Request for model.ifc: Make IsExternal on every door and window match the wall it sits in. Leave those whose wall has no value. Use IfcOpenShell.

First a look at what the model holds.

```python
import ifcopenshell
import ifcopenshell.util.element

model = ifcopenshell.open("model.ifc")
print(model.schema)
seen = {}
for e in model.by_type("IfcDoor") + model.by_type("IfcWindow"):
    if not e.FillsVoids:
        continue
    host = e.FillsVoids[0].RelatingOpeningElement.VoidsElements[0].RelatingBuildingElement
    own = ifcopenshell.util.element.get_pset(e, f"Pset_{e.is_a()[3:].removesuffix('StandardCase')}Common", "IsExternal")
    wall = ifcopenshell.util.element.get_pset(host, "Pset_WallCommon", "IsExternal")
    seen[e.is_a(), own, wall] = seen.get((e.is_a(), own, wall), 0) + 1
for (cls, own, wall), count in sorted(seen.items(), key=str):
    print(count, cls, "IsExternal:", own, "| host wall:", wall)
```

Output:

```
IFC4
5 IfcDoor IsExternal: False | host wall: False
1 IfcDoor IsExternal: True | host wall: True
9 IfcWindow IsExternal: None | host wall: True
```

```python
import ifcopenshell
import ifcopenshell.api.pset
import ifcopenshell.util.element

model = ifcopenshell.open("model.ifc")

count = 0
for ifc_class, pset_name in (("IfcDoor", "Pset_DoorCommon"), ("IfcWindow", "Pset_WindowCommon")):
    for e in model.by_type(ifc_class):
        if not e.FillsVoids:
            continue
        host = e.FillsVoids[0].RelatingOpeningElement.VoidsElements[0].RelatingBuildingElement
        external = ifcopenshell.util.element.get_pset(host, "Pset_WallCommon", "IsExternal")
        if external is None or ifcopenshell.util.element.get_pset(e, pset_name, "IsExternal") == external:
            continue
        pset = ifcopenshell.api.pset.add_pset(model, product=e, name=pset_name)
        ifcopenshell.api.pset.edit_pset(model, pset=pset, properties={"IsExternal": external})
        count += 1

print(count, "updated")

model.write("model_edited.ifc")
```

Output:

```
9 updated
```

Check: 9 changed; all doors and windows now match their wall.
